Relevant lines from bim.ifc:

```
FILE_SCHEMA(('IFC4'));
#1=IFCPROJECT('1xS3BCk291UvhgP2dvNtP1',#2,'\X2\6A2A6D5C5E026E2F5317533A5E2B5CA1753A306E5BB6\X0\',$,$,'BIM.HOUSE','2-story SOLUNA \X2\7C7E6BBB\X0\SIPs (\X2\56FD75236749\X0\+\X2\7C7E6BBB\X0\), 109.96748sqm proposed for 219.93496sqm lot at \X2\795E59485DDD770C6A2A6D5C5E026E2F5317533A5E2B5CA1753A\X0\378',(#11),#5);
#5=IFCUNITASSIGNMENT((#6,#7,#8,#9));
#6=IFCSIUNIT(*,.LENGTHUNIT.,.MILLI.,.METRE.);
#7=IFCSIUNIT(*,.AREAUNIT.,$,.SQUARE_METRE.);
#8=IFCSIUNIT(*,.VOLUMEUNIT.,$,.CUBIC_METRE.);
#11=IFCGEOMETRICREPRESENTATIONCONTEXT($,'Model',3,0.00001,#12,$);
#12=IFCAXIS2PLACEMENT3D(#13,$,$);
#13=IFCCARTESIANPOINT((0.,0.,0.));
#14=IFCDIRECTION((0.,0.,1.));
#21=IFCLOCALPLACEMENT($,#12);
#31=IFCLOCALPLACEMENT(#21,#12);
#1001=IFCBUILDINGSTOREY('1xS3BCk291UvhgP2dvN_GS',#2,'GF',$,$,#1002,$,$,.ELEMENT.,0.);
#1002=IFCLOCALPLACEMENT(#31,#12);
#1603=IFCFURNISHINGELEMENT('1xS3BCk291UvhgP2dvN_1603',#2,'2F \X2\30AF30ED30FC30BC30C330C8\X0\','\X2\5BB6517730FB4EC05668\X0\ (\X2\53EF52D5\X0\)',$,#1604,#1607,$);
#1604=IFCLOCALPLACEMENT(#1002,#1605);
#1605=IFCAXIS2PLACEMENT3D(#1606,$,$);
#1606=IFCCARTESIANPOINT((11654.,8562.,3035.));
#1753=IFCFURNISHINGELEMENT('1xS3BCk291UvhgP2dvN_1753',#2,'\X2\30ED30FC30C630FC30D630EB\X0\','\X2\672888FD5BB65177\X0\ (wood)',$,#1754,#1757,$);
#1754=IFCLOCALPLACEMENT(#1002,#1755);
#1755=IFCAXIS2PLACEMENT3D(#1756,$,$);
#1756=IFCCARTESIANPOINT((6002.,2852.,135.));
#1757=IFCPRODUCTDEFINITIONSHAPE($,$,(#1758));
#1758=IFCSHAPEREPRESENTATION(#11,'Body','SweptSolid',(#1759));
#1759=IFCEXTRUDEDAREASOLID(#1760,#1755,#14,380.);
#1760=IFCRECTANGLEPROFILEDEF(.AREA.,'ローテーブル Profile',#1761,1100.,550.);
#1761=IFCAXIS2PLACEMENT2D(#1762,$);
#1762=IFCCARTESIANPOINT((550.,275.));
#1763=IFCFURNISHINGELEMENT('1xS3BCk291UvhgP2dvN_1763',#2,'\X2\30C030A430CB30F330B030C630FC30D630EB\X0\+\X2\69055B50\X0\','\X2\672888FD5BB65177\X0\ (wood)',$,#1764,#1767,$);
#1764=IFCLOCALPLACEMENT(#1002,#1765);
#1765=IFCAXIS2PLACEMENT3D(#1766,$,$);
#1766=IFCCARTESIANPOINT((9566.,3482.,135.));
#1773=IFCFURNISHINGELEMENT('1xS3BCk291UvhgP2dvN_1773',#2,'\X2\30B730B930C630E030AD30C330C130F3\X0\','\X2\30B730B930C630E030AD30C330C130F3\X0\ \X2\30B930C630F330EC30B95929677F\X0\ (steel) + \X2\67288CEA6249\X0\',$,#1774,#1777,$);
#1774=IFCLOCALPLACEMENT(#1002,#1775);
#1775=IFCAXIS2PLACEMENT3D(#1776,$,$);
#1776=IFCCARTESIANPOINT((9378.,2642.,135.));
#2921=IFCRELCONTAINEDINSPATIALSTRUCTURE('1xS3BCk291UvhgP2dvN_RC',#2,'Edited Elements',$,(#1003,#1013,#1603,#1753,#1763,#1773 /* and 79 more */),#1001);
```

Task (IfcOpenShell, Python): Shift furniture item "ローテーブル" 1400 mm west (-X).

```python
import ifcopenshell
import ifcopenshell.api.geometry
import ifcopenshell.util.placement
import ifcopenshell.util.unit

model = ifcopenshell.open("bim.ifc")
unit_scale = ifcopenshell.util.unit.calculate_unit_scale(model)

item = model.by_guid("1xS3BCk291UvhgP2dvN_1753")
matrix = ifcopenshell.util.placement.get_local_placement(item.ObjectPlacement)
matrix[0, 3] -= 1.4 / unit_scale
ifcopenshell.api.geometry.edit_object_placement(model, product=item, matrix=matrix, is_si=False)

print(ifcopenshell.util.placement.get_local_placement(item.ObjectPlacement).round(3) + 0.0)

model.write("bim_edited.ifc")
```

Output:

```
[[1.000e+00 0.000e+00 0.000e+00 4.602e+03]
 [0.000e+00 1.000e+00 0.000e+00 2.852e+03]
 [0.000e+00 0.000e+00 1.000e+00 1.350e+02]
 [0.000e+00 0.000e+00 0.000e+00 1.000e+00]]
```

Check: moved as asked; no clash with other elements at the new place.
